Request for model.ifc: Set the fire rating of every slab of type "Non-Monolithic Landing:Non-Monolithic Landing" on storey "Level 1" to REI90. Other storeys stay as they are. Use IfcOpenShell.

First a look at what the model holds.

```python
import ifcopenshell
import ifcopenshell.util.element

model = ifcopenshell.open("model.ifc")
print(model.schema)
storey = next(s for s in model.by_type("IfcBuildingStorey") if s.Name == "Level 1")
slabs = [e for e in ifcopenshell.util.element.get_decomposition(storey) if e.is_a("IfcSlab")]
seen = {}
for e in slabs:
    element_type = ifcopenshell.util.element.get_type(e)
    key = (element_type.Name if element_type != e and element_type else None, ifcopenshell.util.element.get_pset(e, "Pset_SlabCommon", "FireRating"))
    seen[key] = seen.get(key, 0) + 1
for (name, value), count in sorted(seen.items(), key=str):
    print(count, "x", name, "|", value)
```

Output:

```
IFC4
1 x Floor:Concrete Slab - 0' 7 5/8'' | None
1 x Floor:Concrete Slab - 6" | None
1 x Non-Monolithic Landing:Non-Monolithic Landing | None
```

```python
import ifcopenshell
import ifcopenshell.api.pset
import ifcopenshell.util.element

model = ifcopenshell.open("model.ifc")

storey = next(s for s in model.by_type("IfcBuildingStorey") if s.Name == "Level 1")
slabs = [e for e in ifcopenshell.util.element.get_decomposition(storey) if e.is_a("IfcSlab")]

count = 0
for e in slabs:
    element_type = ifcopenshell.util.element.get_type(e)
    if element_type in (None, e) or element_type.Name != "Non-Monolithic Landing:Non-Monolithic Landing":
        continue
    # add_pset returns the element's existing set when there is one.
    pset = ifcopenshell.api.pset.add_pset(model, product=e, name="Pset_SlabCommon")
    ifcopenshell.api.pset.edit_pset(model, pset=pset, properties={"FireRating": "REI90"})
    count += 1

print(count, "slabs updated")

model.write("model_rev.ifc")
```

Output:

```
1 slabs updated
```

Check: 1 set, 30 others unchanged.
